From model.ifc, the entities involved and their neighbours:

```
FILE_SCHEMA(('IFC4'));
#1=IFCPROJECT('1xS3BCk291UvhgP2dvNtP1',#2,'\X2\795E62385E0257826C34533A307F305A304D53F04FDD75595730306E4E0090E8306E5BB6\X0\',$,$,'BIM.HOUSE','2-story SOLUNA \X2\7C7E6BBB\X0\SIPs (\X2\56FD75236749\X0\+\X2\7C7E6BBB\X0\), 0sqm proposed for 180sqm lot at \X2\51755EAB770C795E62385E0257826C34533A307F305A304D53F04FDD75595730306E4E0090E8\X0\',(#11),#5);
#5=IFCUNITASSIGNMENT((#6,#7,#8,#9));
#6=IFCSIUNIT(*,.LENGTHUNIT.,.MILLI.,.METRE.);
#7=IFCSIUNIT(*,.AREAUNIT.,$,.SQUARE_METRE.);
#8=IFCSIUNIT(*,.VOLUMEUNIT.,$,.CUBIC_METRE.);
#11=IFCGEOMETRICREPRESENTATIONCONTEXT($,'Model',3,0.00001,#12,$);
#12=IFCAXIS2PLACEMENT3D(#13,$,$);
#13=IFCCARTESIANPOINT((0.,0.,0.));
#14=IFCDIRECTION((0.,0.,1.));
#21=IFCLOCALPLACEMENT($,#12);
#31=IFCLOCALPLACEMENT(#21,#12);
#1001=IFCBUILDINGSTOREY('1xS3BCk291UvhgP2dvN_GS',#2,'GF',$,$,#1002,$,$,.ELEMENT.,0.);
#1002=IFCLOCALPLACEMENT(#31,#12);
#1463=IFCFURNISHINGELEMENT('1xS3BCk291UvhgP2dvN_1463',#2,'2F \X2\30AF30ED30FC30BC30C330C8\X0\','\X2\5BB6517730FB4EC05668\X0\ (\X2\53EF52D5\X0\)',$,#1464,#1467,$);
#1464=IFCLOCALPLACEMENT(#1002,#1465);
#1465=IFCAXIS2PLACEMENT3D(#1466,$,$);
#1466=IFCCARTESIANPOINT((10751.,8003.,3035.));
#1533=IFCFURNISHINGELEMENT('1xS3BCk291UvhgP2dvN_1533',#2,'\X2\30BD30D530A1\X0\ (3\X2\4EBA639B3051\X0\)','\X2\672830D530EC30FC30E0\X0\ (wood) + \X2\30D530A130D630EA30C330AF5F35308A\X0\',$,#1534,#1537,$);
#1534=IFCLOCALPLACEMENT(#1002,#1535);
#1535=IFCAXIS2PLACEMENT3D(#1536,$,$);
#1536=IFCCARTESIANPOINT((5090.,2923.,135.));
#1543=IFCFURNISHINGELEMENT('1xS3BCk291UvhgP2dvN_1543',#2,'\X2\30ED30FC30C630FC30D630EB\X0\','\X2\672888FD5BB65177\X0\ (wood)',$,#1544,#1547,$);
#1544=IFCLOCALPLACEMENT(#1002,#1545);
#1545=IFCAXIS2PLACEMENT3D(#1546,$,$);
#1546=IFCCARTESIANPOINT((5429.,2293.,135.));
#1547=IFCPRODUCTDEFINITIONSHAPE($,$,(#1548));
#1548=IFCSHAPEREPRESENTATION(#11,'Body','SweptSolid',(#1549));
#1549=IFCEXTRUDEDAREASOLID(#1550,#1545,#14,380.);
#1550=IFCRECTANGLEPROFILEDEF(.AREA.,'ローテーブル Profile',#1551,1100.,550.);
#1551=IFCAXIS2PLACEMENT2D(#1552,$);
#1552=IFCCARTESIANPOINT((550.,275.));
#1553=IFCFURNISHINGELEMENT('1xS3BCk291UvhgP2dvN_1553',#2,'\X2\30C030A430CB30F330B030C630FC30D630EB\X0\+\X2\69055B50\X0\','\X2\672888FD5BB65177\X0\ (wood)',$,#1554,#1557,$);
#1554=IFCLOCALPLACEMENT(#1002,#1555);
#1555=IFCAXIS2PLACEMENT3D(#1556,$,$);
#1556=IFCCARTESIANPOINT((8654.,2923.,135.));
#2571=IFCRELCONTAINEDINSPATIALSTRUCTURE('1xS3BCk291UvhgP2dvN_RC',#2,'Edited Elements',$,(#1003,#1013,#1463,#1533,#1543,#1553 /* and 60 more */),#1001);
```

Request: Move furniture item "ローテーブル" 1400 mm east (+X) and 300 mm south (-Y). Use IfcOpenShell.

```python
import ifcopenshell
import ifcopenshell.api.geometry
import ifcopenshell.util.placement
import ifcopenshell.util.unit

model = ifcopenshell.open("model.ifc")
unit_scale = ifcopenshell.util.unit.calculate_unit_scale(model)

item = model.by_guid("1xS3BCk291UvhgP2dvN_1543")
matrix = ifcopenshell.util.placement.get_local_placement(item.ObjectPlacement)
matrix[0, 3] += 1.4 / unit_scale
matrix[1, 3] -= 0.3 / unit_scale
ifcopenshell.api.geometry.edit_object_placement(model, product=item, matrix=matrix, is_si=False)

print(ifcopenshell.util.placement.get_local_placement(item.ObjectPlacement).round(3) + 0.0)

model.write("model_v2.ifc")
```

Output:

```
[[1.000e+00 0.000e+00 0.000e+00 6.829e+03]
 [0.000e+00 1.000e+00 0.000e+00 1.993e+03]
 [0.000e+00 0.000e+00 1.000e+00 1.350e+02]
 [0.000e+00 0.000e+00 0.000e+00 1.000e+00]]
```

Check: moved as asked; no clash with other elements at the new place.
